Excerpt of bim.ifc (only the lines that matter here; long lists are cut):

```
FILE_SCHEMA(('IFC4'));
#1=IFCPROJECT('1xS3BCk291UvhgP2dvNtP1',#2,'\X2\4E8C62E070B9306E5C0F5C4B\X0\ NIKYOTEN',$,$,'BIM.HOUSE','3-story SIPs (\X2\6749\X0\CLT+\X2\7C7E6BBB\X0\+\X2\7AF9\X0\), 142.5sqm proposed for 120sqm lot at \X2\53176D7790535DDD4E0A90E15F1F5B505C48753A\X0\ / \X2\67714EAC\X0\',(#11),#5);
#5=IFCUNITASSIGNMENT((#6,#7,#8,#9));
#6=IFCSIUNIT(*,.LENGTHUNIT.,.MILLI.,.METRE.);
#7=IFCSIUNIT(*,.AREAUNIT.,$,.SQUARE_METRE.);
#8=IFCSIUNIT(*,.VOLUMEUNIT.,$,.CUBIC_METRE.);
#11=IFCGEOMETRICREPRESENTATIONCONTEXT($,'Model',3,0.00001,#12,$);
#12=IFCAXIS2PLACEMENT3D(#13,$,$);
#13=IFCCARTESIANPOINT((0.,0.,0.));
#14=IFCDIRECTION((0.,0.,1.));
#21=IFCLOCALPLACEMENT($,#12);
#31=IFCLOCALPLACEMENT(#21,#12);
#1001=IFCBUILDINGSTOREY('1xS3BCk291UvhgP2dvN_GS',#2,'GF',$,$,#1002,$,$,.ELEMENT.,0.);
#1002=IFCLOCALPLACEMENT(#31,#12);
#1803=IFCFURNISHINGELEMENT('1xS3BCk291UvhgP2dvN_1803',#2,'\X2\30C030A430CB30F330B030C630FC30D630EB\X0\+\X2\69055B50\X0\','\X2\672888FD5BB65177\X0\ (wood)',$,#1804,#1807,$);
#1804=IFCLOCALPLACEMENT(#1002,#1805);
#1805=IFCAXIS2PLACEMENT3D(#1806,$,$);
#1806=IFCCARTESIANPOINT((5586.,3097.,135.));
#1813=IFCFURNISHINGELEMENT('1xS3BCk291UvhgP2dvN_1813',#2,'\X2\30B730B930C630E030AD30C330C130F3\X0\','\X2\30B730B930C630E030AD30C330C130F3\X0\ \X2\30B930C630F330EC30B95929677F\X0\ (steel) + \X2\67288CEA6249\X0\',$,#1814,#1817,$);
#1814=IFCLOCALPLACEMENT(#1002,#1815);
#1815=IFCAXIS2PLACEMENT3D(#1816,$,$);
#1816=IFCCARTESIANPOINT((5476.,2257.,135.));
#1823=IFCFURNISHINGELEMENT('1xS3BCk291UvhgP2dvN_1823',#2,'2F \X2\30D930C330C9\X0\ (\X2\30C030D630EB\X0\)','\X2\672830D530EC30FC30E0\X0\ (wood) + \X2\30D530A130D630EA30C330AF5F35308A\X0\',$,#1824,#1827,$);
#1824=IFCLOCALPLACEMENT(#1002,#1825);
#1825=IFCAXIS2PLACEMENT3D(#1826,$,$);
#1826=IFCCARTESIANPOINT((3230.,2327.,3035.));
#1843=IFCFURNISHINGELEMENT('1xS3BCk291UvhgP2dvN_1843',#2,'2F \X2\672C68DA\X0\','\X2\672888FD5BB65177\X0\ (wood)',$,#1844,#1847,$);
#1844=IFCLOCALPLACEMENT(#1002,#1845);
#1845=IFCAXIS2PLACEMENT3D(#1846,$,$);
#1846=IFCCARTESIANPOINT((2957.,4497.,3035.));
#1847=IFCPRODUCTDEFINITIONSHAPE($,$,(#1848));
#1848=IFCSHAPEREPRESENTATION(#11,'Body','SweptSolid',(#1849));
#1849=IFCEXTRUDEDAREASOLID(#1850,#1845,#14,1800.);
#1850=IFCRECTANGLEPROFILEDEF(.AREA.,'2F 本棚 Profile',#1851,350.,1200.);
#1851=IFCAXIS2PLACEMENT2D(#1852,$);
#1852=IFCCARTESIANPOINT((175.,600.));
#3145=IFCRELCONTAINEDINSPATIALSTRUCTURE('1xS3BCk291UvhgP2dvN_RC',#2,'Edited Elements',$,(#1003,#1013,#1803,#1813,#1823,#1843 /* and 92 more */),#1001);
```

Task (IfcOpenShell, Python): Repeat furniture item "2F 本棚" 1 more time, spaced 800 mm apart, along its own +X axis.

```python
import ifcopenshell
import ifcopenshell.api.geometry
import ifcopenshell.api.root
import ifcopenshell.util.element
import ifcopenshell.util.placement
import ifcopenshell.util.unit

model = ifcopenshell.open("bim.ifc")
unit_scale = ifcopenshell.util.unit.calculate_unit_scale(model)


def reuse_history(source, copy):
    """copy_class also copies each property set's owner history, people and application; keep the originals."""
    for rel in copy.IsDefinedBy:
        if rel.is_a("IfcRelDefinesByProperties") and (history := rel.RelatingPropertyDefinition.OwnerHistory):
            rel.RelatingPropertyDefinition.OwnerHistory = source.OwnerHistory
            ifcopenshell.util.element.remove_deep2(model, history)


source = model.by_guid("1xS3BCk291UvhgP2dvN_1843")
base = ifcopenshell.util.placement.get_local_placement(source.ObjectPlacement)
step = base[:3, 0] * 0.8 / unit_scale

for i in range(1, 2):
    copy = ifcopenshell.api.root.copy_class(model, product=source)
    copy.Representation = ifcopenshell.util.element.copy_deep(
        model, source.Representation, exclude=["IfcGeometricRepresentationContext", "IfcRepresentationMap"]
    )
    reuse_history(source, copy)
    matrix = base.copy()
    matrix[:3, 3] += i * step
    print("added at", matrix[:3, 3].round(3) + 0.0)
    ifcopenshell.api.geometry.edit_object_placement(model, product=copy, matrix=matrix, is_si=False)

model.write("bim_edited.ifc")
```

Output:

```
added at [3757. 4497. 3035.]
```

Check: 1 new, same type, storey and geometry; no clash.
